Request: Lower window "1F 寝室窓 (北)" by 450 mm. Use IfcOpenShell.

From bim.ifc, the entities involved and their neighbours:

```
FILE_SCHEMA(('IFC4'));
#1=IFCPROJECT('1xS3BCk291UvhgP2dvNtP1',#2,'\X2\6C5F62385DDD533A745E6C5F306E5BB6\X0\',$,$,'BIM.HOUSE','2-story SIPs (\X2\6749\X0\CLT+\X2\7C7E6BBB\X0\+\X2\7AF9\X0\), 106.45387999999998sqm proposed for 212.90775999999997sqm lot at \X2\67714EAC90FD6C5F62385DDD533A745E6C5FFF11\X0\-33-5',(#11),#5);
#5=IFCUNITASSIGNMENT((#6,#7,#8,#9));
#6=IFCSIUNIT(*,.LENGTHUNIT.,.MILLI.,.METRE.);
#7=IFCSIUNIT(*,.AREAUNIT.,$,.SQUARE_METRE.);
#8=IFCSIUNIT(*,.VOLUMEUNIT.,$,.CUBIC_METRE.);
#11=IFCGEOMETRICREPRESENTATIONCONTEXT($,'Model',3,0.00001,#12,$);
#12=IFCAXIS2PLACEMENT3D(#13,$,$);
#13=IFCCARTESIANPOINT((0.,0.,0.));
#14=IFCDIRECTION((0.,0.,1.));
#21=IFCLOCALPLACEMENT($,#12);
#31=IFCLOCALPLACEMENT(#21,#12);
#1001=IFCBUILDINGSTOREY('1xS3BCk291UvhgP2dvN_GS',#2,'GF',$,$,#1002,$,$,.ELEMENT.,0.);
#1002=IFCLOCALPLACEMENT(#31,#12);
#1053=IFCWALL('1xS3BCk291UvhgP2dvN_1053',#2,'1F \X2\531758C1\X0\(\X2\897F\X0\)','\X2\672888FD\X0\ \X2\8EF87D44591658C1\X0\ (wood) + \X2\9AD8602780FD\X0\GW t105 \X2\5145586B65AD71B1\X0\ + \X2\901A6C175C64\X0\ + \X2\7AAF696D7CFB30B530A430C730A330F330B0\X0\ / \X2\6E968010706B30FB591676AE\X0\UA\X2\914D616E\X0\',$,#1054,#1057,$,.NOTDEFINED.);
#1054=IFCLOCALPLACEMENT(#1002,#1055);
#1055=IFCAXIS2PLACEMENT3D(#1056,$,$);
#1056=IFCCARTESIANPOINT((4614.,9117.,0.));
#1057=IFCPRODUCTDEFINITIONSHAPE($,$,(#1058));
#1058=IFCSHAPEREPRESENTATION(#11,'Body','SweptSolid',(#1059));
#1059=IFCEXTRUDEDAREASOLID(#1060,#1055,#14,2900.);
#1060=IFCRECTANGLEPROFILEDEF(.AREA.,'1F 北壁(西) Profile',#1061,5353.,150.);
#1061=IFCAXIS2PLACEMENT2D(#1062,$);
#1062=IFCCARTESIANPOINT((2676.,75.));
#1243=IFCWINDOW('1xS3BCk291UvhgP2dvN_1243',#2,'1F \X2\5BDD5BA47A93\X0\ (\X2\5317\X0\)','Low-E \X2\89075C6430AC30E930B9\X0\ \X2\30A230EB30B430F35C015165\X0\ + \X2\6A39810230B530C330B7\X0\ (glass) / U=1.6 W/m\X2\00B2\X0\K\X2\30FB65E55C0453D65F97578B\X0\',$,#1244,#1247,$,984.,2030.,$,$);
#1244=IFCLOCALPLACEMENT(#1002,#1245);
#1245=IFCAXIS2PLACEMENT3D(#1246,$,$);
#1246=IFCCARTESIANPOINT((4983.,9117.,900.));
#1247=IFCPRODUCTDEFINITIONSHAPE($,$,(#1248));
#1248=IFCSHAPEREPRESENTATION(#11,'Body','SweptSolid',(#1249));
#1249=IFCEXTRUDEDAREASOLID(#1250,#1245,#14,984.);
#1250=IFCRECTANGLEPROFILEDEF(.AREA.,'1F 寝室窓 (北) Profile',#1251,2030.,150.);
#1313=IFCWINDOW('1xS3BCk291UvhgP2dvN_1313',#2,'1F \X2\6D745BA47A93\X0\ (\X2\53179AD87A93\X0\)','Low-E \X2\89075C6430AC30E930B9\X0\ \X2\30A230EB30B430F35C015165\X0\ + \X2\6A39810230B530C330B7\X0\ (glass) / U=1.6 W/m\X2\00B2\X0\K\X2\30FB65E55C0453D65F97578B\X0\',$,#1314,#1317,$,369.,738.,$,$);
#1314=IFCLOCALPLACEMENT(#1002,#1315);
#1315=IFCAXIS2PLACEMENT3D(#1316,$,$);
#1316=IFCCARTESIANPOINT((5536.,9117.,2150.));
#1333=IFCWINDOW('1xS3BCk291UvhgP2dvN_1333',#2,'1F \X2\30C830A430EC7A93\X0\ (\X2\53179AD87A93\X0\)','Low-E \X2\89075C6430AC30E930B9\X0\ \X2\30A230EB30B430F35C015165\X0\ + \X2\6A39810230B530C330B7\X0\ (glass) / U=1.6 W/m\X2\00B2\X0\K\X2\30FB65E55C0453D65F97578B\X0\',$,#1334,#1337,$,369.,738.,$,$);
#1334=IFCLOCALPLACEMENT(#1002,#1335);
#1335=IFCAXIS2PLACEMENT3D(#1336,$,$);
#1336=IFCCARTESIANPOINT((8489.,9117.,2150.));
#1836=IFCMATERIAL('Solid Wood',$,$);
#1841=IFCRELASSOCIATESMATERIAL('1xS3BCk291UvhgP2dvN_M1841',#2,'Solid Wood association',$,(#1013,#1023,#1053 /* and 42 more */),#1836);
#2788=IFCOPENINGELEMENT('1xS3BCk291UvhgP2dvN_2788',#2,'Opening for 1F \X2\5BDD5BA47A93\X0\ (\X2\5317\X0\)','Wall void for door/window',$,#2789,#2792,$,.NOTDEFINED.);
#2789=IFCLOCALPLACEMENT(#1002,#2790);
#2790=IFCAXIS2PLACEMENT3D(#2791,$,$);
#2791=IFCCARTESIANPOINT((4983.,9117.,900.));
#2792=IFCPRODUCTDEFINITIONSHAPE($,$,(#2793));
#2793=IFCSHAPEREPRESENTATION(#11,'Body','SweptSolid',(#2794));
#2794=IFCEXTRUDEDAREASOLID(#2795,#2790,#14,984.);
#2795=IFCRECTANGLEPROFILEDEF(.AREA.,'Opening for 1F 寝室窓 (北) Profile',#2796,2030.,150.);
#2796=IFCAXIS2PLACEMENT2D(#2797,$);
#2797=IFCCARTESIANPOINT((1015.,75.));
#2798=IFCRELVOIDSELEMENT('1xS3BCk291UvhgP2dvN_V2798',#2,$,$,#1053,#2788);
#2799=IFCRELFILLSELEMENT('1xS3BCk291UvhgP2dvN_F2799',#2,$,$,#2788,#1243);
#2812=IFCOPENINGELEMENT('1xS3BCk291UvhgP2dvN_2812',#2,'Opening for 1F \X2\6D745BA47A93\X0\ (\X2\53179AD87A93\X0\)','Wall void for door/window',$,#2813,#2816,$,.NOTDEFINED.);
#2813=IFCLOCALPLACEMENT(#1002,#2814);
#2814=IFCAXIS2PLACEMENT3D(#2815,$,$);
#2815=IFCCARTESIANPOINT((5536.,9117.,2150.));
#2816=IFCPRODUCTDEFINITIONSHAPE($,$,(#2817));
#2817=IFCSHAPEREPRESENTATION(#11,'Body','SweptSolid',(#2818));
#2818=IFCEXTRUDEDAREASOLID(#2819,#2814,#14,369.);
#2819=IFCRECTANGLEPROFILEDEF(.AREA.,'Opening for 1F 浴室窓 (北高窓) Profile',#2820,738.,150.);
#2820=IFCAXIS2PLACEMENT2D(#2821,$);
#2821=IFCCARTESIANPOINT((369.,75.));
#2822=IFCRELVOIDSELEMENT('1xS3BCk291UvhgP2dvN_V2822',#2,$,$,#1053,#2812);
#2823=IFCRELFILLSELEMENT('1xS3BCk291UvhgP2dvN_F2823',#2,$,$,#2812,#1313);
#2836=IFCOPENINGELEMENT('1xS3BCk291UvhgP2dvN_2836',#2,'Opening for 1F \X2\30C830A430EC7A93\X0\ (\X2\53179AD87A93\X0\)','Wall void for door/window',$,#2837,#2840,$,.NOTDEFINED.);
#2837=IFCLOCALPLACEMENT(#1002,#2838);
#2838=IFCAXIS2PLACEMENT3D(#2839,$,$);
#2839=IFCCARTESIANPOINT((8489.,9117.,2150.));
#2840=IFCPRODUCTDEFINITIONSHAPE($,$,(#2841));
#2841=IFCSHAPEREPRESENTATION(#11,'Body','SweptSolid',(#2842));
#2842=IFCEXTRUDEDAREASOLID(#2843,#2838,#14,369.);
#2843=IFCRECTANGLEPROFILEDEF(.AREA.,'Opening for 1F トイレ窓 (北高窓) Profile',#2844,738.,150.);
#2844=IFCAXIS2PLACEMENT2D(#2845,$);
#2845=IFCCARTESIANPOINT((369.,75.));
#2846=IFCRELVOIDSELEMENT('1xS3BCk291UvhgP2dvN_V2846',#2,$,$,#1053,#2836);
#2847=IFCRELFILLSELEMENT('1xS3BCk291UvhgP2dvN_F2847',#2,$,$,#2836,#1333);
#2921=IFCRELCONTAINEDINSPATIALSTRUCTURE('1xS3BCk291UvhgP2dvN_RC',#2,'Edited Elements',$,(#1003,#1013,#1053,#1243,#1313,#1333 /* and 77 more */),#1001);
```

```python
import numpy as np
import ifcopenshell
import ifcopenshell.api.geometry
import ifcopenshell.util.placement
import ifcopenshell.util.unit

model = ifcopenshell.open("bim.ifc")
unit_scale = ifcopenshell.util.unit.calculate_unit_scale(model)

window = model.by_guid("1xS3BCk291UvhgP2dvN_1243")
opening = window.FillsVoids[0].RelatingOpeningElement
dz = -450.0

shift = np.array([0.0, 0.0, dz])
# The window is not placed relative to its opening, so move both.
for product in (opening, window):
    matrix = ifcopenshell.util.placement.get_local_placement(product.ObjectPlacement)
    matrix[:3, 3] += shift
    ifcopenshell.api.geometry.edit_object_placement(model, product=product, matrix=matrix, is_si=False)

print(f"moved by {dz * unit_scale:+.3f} m")

model.write("bim_updated.ifc")
```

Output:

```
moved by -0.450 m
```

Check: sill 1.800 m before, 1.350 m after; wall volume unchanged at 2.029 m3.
